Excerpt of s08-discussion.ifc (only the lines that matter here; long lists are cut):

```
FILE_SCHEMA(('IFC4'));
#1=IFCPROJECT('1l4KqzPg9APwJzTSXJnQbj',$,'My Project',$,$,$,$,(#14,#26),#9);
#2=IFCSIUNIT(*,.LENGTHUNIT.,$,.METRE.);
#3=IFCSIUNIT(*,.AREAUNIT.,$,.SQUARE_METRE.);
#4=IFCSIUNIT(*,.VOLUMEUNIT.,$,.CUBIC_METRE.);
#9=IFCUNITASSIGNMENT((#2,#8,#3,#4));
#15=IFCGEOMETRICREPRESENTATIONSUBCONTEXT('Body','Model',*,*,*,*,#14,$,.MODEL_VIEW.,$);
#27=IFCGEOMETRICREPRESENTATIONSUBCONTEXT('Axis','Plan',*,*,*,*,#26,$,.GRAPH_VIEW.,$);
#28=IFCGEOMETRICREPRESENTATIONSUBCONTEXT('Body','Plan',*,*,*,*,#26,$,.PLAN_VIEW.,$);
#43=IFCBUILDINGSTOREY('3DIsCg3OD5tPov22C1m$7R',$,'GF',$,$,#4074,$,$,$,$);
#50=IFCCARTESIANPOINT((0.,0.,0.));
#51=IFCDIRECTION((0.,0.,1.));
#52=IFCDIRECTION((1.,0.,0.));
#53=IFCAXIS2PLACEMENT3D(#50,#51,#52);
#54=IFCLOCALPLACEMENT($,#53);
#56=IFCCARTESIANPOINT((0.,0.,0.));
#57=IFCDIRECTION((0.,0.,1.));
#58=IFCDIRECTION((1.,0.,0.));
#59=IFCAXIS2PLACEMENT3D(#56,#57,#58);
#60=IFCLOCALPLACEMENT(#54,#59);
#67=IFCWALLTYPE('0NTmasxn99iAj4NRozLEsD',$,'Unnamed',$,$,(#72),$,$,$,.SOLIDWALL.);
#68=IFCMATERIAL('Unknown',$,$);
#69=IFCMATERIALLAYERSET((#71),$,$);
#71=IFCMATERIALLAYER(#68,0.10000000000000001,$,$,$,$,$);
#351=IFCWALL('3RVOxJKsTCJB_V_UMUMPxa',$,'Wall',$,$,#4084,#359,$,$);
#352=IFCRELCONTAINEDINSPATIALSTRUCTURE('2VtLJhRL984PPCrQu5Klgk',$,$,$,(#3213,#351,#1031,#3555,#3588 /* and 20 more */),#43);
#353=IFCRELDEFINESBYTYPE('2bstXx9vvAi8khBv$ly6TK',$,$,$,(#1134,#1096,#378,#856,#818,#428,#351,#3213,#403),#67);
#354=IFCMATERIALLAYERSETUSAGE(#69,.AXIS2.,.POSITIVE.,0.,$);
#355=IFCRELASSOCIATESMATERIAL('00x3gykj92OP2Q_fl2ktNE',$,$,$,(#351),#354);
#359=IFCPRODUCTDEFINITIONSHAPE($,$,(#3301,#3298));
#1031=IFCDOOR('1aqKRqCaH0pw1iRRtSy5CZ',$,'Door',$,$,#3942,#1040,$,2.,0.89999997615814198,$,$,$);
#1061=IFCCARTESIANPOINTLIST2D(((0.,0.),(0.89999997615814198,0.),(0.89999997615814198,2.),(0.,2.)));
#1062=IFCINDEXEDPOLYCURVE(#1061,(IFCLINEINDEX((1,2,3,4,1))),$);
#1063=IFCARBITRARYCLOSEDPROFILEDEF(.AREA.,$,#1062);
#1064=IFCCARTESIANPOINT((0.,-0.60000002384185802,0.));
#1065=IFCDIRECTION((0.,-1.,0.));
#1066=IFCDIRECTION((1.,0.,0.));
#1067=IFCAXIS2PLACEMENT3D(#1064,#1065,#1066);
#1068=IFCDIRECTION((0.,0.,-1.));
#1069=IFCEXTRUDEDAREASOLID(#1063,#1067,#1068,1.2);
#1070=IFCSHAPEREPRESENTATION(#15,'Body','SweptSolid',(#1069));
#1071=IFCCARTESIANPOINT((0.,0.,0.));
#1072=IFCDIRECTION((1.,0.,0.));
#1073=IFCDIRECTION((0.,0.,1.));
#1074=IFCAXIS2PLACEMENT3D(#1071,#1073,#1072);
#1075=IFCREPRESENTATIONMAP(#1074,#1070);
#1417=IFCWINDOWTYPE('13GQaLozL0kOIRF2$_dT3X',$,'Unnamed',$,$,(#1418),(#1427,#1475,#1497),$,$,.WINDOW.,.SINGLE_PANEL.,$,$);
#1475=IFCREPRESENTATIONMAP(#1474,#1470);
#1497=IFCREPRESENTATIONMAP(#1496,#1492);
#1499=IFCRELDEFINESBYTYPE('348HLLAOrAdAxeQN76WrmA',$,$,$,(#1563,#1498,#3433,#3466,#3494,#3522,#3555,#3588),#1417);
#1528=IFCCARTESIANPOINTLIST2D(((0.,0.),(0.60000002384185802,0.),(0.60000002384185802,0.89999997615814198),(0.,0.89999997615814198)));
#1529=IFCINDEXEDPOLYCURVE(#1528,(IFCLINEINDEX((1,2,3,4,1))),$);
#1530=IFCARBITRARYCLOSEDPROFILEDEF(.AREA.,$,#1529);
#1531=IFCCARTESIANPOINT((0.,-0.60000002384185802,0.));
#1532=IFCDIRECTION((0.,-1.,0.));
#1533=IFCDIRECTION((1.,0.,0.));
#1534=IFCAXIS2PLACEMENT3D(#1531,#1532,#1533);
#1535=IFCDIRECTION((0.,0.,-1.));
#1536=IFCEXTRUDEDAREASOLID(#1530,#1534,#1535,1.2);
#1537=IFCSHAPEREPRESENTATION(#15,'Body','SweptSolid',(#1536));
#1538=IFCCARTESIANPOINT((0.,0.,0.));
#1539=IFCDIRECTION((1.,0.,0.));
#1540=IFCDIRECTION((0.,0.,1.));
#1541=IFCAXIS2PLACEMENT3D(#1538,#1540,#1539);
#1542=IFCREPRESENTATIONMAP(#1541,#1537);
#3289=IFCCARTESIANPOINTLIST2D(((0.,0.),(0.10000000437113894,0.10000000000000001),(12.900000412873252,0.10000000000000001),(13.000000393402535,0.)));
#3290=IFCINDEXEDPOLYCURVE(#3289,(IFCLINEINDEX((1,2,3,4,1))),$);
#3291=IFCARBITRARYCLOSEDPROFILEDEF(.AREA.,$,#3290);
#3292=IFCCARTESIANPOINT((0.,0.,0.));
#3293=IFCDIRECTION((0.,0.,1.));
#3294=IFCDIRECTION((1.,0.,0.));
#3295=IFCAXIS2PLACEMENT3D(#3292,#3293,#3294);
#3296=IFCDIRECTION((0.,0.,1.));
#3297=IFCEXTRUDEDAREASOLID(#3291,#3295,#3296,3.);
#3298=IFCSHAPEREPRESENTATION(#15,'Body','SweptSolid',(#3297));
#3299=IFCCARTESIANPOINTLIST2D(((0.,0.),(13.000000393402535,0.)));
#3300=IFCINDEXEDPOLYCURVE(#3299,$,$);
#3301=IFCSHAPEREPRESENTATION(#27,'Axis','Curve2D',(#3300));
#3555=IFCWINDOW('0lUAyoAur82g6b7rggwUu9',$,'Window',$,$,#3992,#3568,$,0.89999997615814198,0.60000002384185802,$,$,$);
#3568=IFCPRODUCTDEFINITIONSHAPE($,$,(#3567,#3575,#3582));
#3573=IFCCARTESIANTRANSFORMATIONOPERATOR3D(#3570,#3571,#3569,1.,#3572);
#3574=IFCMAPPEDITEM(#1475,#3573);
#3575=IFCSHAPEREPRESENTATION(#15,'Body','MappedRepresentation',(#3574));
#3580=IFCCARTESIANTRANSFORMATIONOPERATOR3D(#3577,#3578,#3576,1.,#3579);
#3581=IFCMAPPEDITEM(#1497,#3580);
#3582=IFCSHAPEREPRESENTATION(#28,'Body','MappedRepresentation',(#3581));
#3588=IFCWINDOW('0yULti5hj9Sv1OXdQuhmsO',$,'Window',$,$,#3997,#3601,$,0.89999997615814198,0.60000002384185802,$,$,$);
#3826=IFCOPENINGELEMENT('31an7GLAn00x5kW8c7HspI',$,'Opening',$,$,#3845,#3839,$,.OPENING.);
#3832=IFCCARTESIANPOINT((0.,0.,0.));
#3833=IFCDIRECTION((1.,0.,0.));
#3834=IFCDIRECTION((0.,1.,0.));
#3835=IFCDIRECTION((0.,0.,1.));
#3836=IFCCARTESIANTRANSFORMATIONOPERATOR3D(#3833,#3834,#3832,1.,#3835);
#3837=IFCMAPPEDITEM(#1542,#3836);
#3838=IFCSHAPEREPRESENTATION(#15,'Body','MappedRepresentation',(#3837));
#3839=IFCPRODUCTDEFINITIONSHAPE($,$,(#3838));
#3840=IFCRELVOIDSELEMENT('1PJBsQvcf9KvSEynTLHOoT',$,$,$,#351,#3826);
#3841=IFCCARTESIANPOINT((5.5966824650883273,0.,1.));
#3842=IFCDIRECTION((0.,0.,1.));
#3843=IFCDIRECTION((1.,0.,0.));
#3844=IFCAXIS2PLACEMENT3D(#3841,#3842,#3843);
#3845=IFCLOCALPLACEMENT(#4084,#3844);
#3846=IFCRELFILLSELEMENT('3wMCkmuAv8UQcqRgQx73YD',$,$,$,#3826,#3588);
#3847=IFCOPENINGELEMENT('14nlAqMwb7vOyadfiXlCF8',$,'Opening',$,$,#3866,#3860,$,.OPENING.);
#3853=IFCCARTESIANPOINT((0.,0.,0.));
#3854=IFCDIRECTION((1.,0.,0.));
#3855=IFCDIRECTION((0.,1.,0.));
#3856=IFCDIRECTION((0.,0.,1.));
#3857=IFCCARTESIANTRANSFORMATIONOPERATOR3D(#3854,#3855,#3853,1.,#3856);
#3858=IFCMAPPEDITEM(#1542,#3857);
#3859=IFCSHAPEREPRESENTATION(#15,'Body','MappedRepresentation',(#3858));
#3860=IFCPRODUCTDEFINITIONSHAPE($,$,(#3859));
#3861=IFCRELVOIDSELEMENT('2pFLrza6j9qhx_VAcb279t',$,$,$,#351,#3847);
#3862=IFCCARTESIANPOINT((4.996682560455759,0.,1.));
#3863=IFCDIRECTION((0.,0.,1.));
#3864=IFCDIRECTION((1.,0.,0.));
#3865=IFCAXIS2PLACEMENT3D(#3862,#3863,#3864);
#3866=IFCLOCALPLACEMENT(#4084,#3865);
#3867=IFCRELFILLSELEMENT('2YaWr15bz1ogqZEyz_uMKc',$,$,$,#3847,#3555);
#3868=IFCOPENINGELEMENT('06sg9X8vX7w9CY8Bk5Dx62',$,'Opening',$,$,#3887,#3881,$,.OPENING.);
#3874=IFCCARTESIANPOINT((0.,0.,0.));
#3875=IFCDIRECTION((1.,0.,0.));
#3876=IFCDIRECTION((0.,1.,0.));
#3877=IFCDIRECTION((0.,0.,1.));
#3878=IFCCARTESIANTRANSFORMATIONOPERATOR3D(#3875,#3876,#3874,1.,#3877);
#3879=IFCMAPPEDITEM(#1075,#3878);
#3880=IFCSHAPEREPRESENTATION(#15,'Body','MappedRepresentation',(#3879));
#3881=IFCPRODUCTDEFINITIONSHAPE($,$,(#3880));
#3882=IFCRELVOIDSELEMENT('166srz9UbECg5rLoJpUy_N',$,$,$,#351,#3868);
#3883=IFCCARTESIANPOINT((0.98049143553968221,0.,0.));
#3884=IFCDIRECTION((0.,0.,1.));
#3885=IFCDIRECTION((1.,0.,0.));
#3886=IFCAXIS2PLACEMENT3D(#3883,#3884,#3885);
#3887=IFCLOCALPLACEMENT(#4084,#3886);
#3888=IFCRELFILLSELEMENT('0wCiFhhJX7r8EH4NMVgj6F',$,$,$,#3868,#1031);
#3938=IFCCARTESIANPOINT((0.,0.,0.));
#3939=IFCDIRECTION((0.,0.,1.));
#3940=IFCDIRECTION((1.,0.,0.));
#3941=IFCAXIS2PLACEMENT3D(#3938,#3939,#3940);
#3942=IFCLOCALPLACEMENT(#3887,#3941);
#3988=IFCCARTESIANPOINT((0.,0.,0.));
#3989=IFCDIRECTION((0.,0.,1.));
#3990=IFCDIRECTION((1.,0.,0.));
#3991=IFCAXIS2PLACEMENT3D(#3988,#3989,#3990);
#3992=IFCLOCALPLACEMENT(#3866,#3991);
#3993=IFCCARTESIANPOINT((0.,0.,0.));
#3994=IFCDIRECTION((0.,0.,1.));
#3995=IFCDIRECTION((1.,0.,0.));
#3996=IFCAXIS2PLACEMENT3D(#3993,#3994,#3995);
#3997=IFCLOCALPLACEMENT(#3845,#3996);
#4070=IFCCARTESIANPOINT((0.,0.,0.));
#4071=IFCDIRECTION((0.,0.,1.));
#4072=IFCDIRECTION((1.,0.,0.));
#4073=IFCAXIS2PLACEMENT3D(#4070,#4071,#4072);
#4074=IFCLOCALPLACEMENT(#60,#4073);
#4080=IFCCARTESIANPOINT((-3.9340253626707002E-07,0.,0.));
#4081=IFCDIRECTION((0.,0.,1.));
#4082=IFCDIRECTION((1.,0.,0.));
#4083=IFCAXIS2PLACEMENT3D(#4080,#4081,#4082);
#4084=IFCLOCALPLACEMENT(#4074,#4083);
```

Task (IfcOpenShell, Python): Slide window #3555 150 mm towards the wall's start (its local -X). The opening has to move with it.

```python
import ifcopenshell
import ifcopenshell.api.geometry
import ifcopenshell.util.placement
import ifcopenshell.util.unit

model = ifcopenshell.open("s08-discussion.ifc")
unit_scale = ifcopenshell.util.unit.calculate_unit_scale(model)

window = model.by_guid("0lUAyoAur82g6b7rggwUu9")
opening = window.FillsVoids[0].RelatingOpeningElement
wall = opening.VoidsElements[0].RelatingBuildingElement

wall_matrix = ifcopenshell.util.placement.get_local_placement(wall.ObjectPlacement)
shift = wall_matrix[:3, 0] * -0.15 / unit_scale
before = ifcopenshell.util.placement.get_local_placement(window.ObjectPlacement)[:3, 3].copy()

# The window is placed relative to its opening, so it follows when the opening moves.
matrix = ifcopenshell.util.placement.get_local_placement(opening.ObjectPlacement)
matrix[:3, 3] += shift
ifcopenshell.api.geometry.edit_object_placement(
    model, product=opening, matrix=matrix, is_si=False, should_transform_children=True
)

after = ifcopenshell.util.placement.get_local_placement(window.ObjectPlacement)[:3, 3]
print("window moved by", (after - before).round(3) + 0.0)

model.write("s08-discussion_edited.ifc")
```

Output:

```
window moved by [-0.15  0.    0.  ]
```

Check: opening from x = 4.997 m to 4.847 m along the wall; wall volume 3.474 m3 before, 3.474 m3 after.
